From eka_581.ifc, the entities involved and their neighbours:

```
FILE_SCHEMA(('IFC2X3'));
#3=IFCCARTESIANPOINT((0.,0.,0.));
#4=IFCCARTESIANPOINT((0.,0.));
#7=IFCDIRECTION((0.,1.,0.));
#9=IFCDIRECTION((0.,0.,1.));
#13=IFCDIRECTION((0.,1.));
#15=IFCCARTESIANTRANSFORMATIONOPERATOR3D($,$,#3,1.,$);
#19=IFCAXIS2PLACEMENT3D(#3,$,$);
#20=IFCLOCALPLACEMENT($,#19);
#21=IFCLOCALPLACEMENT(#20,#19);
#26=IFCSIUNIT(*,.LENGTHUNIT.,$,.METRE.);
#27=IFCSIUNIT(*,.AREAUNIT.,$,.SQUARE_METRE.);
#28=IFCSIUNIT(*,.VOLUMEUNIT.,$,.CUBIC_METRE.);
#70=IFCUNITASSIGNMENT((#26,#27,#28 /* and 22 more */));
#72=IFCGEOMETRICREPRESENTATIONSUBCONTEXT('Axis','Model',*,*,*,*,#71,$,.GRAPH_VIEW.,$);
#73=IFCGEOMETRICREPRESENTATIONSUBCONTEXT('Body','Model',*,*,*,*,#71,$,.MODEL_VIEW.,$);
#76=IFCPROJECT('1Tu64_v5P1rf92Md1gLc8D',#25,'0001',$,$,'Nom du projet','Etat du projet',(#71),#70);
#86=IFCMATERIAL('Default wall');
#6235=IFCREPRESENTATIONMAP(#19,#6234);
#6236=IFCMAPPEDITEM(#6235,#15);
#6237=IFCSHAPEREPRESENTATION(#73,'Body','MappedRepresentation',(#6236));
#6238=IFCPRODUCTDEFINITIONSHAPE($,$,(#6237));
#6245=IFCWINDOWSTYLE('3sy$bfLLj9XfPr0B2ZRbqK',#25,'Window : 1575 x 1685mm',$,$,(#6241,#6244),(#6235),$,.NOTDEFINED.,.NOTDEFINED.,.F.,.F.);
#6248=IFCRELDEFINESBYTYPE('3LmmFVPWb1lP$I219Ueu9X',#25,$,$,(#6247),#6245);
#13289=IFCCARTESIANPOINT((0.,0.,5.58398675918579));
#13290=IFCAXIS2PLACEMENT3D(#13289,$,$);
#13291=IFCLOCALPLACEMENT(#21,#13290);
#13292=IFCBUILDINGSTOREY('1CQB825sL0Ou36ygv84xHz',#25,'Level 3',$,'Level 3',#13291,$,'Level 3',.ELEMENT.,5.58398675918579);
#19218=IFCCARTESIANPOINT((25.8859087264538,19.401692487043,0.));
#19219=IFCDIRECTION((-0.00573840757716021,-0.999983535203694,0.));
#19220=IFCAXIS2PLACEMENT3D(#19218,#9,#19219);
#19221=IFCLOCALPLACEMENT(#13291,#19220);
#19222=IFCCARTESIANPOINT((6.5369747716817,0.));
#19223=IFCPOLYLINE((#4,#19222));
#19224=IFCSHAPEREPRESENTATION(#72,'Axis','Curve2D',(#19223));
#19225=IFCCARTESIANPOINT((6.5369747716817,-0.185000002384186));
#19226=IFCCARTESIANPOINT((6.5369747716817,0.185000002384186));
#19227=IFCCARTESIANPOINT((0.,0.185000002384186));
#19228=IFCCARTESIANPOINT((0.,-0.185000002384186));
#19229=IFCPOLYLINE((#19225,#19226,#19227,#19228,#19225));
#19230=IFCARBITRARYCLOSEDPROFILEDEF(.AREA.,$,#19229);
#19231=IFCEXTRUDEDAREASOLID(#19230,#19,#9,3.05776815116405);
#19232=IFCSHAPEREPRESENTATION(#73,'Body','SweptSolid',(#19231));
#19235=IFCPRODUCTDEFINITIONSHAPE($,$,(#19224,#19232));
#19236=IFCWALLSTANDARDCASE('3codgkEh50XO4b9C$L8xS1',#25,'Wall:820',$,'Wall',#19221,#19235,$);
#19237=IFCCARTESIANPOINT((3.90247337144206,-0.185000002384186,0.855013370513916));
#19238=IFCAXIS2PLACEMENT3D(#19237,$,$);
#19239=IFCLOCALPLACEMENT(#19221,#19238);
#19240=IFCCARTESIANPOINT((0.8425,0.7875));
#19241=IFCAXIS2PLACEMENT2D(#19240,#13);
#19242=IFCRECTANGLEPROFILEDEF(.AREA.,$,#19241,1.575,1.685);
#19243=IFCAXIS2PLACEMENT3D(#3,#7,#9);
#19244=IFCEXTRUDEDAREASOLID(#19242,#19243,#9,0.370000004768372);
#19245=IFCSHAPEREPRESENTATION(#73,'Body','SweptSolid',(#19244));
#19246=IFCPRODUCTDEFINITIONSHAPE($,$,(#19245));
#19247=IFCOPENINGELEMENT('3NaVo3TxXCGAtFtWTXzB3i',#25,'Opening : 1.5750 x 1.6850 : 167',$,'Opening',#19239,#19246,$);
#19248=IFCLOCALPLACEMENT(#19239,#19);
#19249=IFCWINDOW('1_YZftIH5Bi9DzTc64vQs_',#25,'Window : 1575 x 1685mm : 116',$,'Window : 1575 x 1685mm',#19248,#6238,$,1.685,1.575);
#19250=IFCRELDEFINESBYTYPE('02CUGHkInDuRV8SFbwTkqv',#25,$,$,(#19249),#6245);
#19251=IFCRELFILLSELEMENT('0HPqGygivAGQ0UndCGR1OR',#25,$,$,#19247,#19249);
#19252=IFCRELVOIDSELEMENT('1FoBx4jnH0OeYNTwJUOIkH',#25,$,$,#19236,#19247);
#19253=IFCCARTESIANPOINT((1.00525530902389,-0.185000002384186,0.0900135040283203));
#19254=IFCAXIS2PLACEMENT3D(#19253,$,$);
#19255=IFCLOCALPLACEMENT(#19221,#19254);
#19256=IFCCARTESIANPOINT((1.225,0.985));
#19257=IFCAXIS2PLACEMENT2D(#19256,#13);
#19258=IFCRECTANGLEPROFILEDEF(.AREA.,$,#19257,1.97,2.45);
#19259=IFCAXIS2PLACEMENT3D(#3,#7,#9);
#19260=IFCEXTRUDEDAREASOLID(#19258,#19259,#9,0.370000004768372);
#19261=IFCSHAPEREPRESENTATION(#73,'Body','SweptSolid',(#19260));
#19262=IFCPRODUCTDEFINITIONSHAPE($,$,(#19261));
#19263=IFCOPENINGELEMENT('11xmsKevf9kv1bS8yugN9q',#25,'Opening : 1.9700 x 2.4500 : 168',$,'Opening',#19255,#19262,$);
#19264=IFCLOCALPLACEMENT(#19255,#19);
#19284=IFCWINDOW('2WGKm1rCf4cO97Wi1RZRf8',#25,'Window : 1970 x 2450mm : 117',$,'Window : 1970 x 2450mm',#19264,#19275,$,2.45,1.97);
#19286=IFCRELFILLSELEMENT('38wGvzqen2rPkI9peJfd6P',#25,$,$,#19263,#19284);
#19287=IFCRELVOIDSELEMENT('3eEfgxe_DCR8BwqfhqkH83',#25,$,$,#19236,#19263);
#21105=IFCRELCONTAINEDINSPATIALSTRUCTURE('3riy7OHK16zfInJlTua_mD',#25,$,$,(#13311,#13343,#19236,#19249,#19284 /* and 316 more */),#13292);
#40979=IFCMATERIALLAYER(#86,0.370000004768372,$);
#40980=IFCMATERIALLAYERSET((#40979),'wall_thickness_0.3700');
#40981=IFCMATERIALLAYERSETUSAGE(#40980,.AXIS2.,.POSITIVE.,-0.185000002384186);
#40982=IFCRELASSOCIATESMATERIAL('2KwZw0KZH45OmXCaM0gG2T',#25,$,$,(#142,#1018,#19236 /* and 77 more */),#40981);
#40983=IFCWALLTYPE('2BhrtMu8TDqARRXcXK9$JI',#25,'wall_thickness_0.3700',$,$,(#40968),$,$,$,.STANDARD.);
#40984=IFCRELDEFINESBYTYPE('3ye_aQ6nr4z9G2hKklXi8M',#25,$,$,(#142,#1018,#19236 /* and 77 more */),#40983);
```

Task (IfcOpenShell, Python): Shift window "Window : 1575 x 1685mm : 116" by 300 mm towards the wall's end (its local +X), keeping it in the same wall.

```python
import ifcopenshell
import ifcopenshell.api.geometry
import ifcopenshell.util.placement

model = ifcopenshell.open("eka_581.ifc")

window = model.by_guid("1_YZftIH5Bi9DzTc64vQs_")
opening = window.FillsVoids[0].RelatingOpeningElement
wall = opening.VoidsElements[0].RelatingBuildingElement

wall_matrix = ifcopenshell.util.placement.get_local_placement(wall.ObjectPlacement)
shift = wall_matrix[:3, 0] * 0.3
before = ifcopenshell.util.placement.get_local_placement(window.ObjectPlacement)[:3, 3].copy()

# The window is placed relative to its opening, so it follows when the opening moves.
matrix = ifcopenshell.util.placement.get_local_placement(opening.ObjectPlacement)
matrix[:3, 3] += shift
ifcopenshell.api.geometry.edit_object_placement(
    model, product=opening, matrix=matrix, is_si=False, should_transform_children=True
)

after = ifcopenshell.util.placement.get_local_placement(window.ObjectPlacement)[:3, 3]
print("window moved by", (after - before).round(3) + 0.0)

model.write("eka_581-out.ifc")
```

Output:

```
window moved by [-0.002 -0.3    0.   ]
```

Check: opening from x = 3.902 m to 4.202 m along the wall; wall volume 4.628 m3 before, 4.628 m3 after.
